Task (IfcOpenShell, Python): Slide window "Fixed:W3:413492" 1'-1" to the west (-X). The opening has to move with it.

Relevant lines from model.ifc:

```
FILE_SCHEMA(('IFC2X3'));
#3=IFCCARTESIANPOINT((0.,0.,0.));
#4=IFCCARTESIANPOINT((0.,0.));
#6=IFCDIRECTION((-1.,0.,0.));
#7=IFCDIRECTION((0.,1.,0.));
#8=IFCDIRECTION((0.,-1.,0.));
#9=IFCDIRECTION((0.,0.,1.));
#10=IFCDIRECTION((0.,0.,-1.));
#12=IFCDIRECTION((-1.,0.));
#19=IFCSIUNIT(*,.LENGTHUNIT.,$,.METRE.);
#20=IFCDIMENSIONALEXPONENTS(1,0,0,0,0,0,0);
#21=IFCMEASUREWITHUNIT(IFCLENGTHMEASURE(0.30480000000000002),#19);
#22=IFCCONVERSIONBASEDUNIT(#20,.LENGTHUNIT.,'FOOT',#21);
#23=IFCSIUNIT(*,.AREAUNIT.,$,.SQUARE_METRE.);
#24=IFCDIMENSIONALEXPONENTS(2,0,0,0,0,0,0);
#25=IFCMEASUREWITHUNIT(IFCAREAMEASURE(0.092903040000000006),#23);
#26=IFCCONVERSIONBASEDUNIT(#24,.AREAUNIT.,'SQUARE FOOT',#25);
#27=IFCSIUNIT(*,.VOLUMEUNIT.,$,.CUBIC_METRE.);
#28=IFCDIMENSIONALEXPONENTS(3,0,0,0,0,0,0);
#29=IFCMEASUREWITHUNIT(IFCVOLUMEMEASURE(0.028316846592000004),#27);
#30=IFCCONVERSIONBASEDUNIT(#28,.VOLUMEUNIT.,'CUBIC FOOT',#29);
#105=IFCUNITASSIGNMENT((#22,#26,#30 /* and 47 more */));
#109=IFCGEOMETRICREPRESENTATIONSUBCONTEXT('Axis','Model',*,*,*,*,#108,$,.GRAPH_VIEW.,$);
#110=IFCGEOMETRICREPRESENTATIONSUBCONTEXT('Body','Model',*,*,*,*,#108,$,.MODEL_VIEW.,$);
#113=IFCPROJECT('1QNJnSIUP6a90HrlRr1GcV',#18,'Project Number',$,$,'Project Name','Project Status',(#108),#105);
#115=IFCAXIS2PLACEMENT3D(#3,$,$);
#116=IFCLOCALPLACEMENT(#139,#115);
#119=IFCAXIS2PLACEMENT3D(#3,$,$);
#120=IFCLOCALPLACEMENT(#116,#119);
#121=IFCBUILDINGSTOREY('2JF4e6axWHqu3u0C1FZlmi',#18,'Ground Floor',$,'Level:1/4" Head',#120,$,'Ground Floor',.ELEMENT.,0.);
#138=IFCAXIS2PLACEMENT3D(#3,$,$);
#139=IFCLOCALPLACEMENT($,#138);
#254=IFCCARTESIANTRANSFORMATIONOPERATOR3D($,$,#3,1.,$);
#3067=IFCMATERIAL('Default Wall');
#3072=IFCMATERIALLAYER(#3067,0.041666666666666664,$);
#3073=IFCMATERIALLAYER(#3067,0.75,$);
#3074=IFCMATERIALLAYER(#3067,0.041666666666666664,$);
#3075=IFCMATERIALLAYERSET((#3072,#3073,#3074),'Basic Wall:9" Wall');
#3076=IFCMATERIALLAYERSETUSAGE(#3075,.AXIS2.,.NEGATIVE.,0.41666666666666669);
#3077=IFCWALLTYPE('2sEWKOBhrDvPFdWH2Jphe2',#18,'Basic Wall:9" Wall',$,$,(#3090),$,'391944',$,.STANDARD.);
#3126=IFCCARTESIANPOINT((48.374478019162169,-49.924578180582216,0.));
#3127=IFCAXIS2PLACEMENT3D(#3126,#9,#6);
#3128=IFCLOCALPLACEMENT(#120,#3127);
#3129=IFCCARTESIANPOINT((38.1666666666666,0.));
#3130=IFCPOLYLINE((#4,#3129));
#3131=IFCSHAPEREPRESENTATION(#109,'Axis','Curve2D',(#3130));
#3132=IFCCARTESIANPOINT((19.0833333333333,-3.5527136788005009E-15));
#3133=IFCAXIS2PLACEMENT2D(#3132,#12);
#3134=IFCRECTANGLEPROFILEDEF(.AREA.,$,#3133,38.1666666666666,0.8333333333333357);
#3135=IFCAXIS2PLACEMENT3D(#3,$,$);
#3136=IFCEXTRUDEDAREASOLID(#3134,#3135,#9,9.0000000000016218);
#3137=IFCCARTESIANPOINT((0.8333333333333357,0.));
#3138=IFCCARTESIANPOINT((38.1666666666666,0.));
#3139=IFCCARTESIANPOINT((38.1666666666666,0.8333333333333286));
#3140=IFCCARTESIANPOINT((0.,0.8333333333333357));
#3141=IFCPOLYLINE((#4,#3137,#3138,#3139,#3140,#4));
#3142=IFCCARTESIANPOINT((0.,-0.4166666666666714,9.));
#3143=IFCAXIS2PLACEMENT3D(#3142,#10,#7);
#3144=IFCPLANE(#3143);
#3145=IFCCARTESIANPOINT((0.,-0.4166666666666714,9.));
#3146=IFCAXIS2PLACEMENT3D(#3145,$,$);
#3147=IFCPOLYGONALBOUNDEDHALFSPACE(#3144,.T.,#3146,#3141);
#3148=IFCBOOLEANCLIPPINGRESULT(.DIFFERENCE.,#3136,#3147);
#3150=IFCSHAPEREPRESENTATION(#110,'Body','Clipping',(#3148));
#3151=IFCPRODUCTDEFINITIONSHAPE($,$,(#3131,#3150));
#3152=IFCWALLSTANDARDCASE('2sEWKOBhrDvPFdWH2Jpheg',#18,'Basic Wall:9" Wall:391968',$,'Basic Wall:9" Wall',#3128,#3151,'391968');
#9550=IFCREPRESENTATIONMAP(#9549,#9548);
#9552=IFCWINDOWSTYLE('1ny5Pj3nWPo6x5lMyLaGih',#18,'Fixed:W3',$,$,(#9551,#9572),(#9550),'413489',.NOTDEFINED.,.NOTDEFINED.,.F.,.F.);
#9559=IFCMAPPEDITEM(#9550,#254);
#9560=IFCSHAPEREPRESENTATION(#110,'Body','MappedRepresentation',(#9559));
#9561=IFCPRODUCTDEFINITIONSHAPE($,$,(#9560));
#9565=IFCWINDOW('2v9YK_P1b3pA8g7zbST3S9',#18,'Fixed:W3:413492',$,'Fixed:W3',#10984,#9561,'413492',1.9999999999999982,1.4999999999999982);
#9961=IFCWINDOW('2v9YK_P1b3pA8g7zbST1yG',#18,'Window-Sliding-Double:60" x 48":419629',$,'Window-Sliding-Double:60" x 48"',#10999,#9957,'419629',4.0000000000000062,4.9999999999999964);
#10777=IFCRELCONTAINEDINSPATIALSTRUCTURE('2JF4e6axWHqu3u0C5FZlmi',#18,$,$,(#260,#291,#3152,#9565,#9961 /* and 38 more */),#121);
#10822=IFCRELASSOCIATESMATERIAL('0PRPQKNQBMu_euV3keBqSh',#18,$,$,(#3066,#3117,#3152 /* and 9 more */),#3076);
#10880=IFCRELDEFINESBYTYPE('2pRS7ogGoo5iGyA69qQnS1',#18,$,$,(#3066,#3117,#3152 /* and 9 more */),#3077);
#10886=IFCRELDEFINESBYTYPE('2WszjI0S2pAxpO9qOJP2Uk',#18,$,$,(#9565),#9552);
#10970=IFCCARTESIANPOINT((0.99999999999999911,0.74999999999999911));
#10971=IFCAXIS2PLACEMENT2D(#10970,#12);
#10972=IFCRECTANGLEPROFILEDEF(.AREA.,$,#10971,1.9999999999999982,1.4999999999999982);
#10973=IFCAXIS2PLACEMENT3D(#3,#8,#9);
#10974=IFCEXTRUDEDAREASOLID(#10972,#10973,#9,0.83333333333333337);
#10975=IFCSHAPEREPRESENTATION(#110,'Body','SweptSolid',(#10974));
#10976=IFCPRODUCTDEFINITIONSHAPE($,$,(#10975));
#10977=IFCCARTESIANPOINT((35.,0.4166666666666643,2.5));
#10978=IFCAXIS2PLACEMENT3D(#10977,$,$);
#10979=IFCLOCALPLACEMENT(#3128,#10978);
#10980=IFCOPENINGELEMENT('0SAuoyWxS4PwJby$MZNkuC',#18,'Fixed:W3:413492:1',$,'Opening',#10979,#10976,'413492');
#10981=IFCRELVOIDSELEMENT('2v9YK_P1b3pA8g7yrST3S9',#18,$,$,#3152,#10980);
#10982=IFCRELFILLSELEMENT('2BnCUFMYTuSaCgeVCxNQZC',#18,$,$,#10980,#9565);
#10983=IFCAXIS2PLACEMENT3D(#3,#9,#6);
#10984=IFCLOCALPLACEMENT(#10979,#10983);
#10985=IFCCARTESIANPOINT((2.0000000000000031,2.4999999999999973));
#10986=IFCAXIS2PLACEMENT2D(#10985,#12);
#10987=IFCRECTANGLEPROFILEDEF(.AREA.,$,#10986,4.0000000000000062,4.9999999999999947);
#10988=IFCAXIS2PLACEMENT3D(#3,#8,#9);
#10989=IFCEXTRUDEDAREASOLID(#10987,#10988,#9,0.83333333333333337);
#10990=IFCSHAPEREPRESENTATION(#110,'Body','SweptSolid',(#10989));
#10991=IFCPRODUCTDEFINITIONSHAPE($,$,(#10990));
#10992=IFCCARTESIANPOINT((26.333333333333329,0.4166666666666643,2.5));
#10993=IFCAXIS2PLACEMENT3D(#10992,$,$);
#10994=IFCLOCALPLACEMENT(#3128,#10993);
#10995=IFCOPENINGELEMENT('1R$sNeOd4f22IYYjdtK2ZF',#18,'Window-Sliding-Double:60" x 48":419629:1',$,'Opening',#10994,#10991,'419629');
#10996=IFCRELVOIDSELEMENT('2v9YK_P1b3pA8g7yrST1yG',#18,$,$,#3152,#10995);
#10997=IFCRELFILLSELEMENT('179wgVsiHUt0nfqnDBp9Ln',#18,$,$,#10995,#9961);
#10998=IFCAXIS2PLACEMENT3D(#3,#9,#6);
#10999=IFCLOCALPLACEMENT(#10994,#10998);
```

```python
import ifcopenshell
import ifcopenshell.api.geometry
import ifcopenshell.util.placement
import ifcopenshell.util.unit

model = ifcopenshell.open("model.ifc")
unit_scale = ifcopenshell.util.unit.calculate_unit_scale(model)

window = model.by_id(9565)
opening = window.FillsVoids[0].RelatingOpeningElement
wall = opening.VoidsElements[0].RelatingBuildingElement

wall_matrix = ifcopenshell.util.placement.get_local_placement(wall.ObjectPlacement)
shift = wall_matrix[:3, 0] * 13 * 0.0254 / unit_scale
before = ifcopenshell.util.placement.get_local_placement(window.ObjectPlacement)[:3, 3].copy()

# The window is placed relative to its opening, so it follows when the opening moves.
matrix = ifcopenshell.util.placement.get_local_placement(opening.ObjectPlacement)
matrix[:3, 3] += shift
ifcopenshell.api.geometry.edit_object_placement(
    model, product=opening, matrix=matrix, is_si=False, should_transform_children=True
)

after = ifcopenshell.util.placement.get_local_placement(window.ObjectPlacement)[:3, 3]
print("window moved by", (after - before).round(3) + 0.0)

model.write("model-out.ifc")
```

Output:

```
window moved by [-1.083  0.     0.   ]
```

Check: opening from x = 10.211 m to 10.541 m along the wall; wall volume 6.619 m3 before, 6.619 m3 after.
